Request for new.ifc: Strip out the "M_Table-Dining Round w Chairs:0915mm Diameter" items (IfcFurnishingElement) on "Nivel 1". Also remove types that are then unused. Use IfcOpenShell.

First a look at what the model holds.

```python
import ifcopenshell
import ifcopenshell.util.element

model = ifcopenshell.open("new.ifc")
print(model.schema)
storey = next(s for s in model.by_type("IfcBuildingStorey") if s.Name == "Nivel 1")
furniture = [e for e in ifcopenshell.util.element.get_decomposition(storey) if e.is_a("IfcFurnishingElement")]
seen = {}
for e in furniture:
    element_type = ifcopenshell.util.element.get_type(e)
    name = element_type.Name if element_type not in (None, e) else None
    seen[name] = seen.get(name, 0) + 1
for name, count in sorted(seen.items(), key=str):
    print(count, "x", name)
```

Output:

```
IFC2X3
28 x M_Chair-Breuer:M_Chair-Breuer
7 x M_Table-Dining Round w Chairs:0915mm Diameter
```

```python
import ifcopenshell
import ifcopenshell.api.root
import ifcopenshell.util.element

model = ifcopenshell.open("new.ifc")

storey = next(s for s in model.by_type("IfcBuildingStorey") if s.Name == "Nivel 1")
furniture = [e for e in ifcopenshell.util.element.get_decomposition(storey) if e.is_a("IfcFurnishingElement")]
targets = [e for e in furniture if (t := ifcopenshell.util.element.get_type(e)) not in (None, e) and t.Name == "M_Table-Dining Round w Chairs:0915mm Diameter"]
types = {ifcopenshell.util.element.get_type(e) for e in targets} - {None, *targets}

for e in targets:
    ifcopenshell.api.root.remove_product(model, product=e)
print(len(targets), "removed")

unused = [t for t in types if not ifcopenshell.util.element.get_types(t)]
for t in unused:
    ifcopenshell.api.root.remove_product(model, product=t)
print(len(unused), "unused types removed")

model.write("new_rev.ifc")
```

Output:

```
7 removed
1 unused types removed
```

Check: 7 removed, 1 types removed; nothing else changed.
